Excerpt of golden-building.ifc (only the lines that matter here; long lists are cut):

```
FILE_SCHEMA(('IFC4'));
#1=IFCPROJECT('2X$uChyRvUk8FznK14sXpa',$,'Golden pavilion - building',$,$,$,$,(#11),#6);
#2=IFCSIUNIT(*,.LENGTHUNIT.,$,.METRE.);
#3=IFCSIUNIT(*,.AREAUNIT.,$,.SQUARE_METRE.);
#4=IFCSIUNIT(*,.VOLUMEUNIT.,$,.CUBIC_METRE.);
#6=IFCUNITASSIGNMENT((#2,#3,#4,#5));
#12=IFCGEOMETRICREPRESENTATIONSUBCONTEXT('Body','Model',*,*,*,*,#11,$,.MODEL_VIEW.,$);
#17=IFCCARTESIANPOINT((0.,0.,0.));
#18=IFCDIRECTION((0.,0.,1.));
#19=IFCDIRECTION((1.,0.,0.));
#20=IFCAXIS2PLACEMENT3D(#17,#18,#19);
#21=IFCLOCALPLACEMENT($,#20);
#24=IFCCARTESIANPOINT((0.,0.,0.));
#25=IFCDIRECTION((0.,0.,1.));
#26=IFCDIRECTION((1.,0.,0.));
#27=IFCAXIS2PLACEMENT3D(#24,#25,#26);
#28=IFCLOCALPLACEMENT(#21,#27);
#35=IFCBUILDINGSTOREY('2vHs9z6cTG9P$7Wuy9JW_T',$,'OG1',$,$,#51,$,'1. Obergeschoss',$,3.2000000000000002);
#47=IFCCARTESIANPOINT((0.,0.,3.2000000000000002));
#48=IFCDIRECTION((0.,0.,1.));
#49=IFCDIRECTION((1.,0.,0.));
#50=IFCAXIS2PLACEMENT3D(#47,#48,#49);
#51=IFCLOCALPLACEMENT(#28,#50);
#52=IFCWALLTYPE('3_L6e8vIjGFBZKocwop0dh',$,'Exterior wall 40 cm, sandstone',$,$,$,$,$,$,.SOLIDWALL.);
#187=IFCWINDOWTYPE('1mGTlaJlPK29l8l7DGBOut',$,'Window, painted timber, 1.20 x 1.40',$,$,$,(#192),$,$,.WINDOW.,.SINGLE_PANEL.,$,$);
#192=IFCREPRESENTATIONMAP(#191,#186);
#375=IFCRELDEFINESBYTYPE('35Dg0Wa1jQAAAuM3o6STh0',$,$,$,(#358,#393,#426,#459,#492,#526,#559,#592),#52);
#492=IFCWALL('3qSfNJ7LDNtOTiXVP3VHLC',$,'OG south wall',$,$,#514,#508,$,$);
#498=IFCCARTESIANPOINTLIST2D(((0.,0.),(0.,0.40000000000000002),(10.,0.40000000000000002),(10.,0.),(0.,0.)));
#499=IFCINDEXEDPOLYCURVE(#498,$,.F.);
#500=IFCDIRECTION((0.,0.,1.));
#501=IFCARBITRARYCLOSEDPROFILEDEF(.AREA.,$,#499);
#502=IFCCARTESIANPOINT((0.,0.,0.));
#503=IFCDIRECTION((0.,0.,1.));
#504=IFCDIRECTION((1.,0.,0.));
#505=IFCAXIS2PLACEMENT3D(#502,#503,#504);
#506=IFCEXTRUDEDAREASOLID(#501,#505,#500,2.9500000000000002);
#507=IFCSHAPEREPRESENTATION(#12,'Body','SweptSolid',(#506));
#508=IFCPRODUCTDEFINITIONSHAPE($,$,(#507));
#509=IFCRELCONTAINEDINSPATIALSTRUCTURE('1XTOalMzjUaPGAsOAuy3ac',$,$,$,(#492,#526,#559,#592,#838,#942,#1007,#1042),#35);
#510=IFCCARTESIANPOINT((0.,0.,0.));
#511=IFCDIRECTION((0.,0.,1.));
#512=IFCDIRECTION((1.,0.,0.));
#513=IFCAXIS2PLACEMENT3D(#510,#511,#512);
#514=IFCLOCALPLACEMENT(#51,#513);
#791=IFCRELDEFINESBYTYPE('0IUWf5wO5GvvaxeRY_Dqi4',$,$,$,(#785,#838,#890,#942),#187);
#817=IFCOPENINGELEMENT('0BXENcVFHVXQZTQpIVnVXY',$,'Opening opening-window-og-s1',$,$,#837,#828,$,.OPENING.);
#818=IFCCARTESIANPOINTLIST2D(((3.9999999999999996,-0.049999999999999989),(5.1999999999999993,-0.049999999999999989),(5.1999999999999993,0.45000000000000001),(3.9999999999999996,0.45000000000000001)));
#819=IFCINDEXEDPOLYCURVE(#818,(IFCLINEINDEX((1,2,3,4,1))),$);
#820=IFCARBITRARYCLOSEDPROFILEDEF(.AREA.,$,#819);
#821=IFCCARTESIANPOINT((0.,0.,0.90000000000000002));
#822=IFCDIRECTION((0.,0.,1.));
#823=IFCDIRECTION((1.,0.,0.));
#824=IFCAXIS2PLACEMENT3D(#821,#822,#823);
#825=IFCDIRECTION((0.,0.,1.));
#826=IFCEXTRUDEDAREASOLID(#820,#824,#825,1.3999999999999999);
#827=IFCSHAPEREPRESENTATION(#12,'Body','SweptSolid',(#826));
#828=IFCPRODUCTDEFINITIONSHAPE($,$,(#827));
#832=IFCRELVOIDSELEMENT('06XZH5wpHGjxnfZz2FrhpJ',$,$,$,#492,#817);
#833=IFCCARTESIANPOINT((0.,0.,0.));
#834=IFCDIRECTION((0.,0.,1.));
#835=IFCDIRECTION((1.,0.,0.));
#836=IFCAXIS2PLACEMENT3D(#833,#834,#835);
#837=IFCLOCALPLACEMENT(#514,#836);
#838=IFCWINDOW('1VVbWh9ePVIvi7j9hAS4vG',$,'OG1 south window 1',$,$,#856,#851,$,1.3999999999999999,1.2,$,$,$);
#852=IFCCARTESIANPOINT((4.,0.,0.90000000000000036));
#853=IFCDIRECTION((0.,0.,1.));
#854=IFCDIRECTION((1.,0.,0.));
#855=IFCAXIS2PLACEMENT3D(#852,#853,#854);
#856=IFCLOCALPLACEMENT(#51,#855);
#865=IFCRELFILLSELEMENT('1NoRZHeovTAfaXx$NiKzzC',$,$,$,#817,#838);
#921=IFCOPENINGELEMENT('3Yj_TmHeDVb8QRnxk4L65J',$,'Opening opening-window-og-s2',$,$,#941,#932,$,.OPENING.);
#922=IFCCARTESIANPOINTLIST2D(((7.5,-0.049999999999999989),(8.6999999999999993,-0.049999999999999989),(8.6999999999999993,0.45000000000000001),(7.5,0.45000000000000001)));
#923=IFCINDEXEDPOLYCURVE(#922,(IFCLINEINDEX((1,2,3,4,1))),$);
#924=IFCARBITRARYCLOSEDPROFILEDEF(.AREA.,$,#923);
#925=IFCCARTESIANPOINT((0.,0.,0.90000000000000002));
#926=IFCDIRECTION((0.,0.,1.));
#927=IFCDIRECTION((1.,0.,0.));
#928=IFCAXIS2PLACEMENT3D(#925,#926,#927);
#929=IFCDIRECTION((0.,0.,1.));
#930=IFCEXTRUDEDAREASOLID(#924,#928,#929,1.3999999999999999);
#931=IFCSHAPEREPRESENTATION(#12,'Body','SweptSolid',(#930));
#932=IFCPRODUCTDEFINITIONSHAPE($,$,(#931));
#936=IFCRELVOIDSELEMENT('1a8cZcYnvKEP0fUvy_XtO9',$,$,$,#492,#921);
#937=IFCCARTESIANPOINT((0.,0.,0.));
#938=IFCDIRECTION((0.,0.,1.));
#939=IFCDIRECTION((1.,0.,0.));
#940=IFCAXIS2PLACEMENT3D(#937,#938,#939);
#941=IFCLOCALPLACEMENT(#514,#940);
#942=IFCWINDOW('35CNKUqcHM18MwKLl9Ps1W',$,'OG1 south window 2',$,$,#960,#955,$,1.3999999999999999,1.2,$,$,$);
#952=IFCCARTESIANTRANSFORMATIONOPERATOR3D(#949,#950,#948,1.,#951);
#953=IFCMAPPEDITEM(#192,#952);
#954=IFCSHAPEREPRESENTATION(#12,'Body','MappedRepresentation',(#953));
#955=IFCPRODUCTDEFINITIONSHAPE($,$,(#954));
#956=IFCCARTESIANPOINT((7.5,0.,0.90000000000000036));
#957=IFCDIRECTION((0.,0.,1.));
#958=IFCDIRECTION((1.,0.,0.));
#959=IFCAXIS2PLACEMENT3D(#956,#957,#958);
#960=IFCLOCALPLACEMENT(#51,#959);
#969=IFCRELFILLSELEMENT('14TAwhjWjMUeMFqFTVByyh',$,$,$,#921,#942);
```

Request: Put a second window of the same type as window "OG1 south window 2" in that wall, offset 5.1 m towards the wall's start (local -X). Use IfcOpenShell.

```python
import ifcopenshell
import ifcopenshell.api.feature
import ifcopenshell.api.geometry
import ifcopenshell.api.root
import ifcopenshell.geom
import ifcopenshell.util.element
import ifcopenshell.util.placement
import ifcopenshell.util.shape
import ifcopenshell.util.unit

model = ifcopenshell.open("golden-building.ifc")
unit_scale = ifcopenshell.util.unit.calculate_unit_scale(model)
settings = ifcopenshell.geom.settings()


def volume(element):
    """Net volume in cubic metres, openings subtracted."""
    shape = ifcopenshell.geom.create_shape(settings, element)
    return ifcopenshell.util.shape.get_volume(shape.geometry)


window = model.by_guid("35CNKUqcHM18MwKLl9Ps1W")
opening = window.FillsVoids[0].RelatingOpeningElement
wall = opening.VoidsElements[0].RelatingBuildingElement
before = volume(wall)
shift = ifcopenshell.util.placement.get_local_placement(wall.ObjectPlacement)[:3, 0] * -5.1 / unit_scale

# copy_class copies the void relationship, type, container and properties, but no geometry.
new_opening = ifcopenshell.api.root.copy_class(model, product=opening)
new_opening.Representation = ifcopenshell.util.element.copy_deep(
    model, opening.Representation, exclude=["IfcGeometricRepresentationContext", "IfcRepresentationMap"]
)
new_window = ifcopenshell.api.root.copy_class(model, product=window)
new_window.Representation = ifcopenshell.util.element.copy_deep(
    model, window.Representation, exclude=["IfcGeometricRepresentationContext", "IfcRepresentationMap"]
)
ifcopenshell.api.feature.add_filling(model, opening=new_opening, element=new_window)

for old, new in ((opening, new_opening), (window, new_window)):
    matrix = ifcopenshell.util.placement.get_local_placement(old.ObjectPlacement)
    matrix[:3, 3] += shift
    ifcopenshell.api.geometry.edit_object_placement(model, product=new, matrix=matrix, is_si=False)

after = volume(wall)

print(f"wall volume {before:.3f} -> {after:.3f} m3")

model.write("golden-building_rev.ifc")
```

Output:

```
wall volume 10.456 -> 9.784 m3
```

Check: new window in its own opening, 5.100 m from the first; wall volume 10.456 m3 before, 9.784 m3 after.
